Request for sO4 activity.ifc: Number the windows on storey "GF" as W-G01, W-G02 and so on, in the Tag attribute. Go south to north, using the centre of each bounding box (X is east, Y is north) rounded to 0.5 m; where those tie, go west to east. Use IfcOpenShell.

First a look at what the model holds.

```python
import ifcopenshell
import ifcopenshell.util.element
import ifcopenshell.util.placement

model = ifcopenshell.open("sO4 activity.ifc")
print(model.schema)
storey = next(s for s in model.by_type("IfcBuildingStorey") if s.Name == "GF")
windows = [e for e in ifcopenshell.util.element.get_decomposition(storey) if e.is_a("IfcWindow")]
for e in sorted(windows, key=lambda e: e.id()):
    origin = ifcopenshell.util.placement.get_local_placement(e.ObjectPlacement)[:3, 3]
    print(e.id(), e.Tag, e.Name, origin.round(2) + 0.0, sep=" | ")
```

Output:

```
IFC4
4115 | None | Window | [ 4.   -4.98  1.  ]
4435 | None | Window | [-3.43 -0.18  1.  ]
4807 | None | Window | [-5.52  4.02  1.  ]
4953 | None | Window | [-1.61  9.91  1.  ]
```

```python
import ifcopenshell
import ifcopenshell.geom
import ifcopenshell.util.element
import ifcopenshell.util.shape

model = ifcopenshell.open("sO4 activity.ifc")
settings = ifcopenshell.geom.settings()
settings.set("use-world-coords", True)


def centre(element):
    shape = ifcopenshell.geom.create_shape(settings, element)
    return ifcopenshell.util.shape.get_bbox_centroid(shape.geometry)


storey = next(s for s in model.by_type("IfcBuildingStorey") if s.Name == "GF")
windows = [e for e in ifcopenshell.util.element.get_decomposition(storey) if e.is_a("IfcWindow")]

# Insertion points can sit at a corner or the storey origin, so sort by the geometry (in metres).
centres = {e: centre(e) for e in windows}
windows.sort(key=lambda e: (round(centres[e][1] / 0.5), centres[e][0]))

for i, e in enumerate(windows, start=1):
    number = f"W-G{i:02d}"
    e.Tag = number
    print(e.id(), number)

model.write("sO4 activity_updated.ifc")
```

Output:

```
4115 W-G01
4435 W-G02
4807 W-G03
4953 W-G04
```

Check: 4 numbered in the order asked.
